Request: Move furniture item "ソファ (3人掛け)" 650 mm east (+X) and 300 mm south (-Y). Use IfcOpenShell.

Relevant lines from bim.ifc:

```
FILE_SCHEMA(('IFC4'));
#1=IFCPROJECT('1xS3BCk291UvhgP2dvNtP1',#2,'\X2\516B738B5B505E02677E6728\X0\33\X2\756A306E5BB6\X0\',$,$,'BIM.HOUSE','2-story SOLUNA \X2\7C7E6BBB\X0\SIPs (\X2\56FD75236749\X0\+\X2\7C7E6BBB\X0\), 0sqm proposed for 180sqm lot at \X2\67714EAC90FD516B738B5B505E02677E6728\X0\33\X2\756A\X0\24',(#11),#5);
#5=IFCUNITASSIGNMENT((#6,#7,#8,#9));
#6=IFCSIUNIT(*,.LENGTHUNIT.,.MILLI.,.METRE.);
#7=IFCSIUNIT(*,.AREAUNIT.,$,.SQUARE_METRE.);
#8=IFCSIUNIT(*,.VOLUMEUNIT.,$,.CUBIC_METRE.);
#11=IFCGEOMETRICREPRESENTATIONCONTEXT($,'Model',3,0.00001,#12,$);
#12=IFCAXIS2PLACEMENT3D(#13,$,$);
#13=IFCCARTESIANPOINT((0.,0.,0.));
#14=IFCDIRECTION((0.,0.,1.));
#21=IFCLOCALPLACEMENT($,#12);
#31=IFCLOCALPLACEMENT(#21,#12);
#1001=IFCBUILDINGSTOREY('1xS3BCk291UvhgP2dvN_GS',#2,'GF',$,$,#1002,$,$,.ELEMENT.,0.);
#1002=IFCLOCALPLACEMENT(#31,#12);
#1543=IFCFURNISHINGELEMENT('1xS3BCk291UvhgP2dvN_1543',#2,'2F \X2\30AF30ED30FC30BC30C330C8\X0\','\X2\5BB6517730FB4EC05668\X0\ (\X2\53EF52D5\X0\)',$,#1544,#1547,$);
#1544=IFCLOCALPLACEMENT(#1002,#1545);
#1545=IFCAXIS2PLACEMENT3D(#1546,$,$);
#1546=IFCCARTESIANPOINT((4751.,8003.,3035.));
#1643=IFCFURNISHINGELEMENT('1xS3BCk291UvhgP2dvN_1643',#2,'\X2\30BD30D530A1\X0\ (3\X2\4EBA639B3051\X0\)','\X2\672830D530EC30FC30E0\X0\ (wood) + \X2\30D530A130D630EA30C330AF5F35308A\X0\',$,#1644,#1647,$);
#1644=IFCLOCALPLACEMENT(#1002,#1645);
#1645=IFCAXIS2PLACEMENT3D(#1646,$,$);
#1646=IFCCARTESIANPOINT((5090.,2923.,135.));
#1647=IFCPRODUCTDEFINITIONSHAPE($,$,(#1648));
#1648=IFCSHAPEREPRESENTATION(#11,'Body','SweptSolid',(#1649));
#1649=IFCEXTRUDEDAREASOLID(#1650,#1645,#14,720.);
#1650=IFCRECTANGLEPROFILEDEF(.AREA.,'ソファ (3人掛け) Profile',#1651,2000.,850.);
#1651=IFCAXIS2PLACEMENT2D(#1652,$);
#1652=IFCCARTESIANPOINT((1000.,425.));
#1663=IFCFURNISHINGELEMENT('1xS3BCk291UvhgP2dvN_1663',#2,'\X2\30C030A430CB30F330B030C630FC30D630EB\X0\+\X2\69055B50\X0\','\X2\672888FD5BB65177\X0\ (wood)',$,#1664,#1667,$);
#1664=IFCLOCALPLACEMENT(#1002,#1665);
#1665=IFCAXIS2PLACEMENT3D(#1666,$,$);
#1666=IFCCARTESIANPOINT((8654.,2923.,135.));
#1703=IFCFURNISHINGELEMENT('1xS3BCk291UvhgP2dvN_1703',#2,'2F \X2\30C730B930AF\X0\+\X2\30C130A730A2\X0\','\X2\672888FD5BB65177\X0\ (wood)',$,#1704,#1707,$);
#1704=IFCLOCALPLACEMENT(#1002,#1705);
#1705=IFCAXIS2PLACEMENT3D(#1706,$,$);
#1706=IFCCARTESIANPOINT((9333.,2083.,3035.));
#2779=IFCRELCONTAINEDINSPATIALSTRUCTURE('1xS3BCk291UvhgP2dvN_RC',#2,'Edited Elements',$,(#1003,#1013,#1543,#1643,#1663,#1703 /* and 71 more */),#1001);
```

```python
import ifcopenshell
import ifcopenshell.api.geometry
import ifcopenshell.util.placement
import ifcopenshell.util.unit

model = ifcopenshell.open("bim.ifc")
unit_scale = ifcopenshell.util.unit.calculate_unit_scale(model)

item = model.by_guid("1xS3BCk291UvhgP2dvN_1643")
matrix = ifcopenshell.util.placement.get_local_placement(item.ObjectPlacement)
matrix[0, 3] += 0.65 / unit_scale
matrix[1, 3] -= 0.3 / unit_scale
ifcopenshell.api.geometry.edit_object_placement(model, product=item, matrix=matrix, is_si=False)

print(ifcopenshell.util.placement.get_local_placement(item.ObjectPlacement).round(3) + 0.0)

model.write("bim_edited.ifc")
```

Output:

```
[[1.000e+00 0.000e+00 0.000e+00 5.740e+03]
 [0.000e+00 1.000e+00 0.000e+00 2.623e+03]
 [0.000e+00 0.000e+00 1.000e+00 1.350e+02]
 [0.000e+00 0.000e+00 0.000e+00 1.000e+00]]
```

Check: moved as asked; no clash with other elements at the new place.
